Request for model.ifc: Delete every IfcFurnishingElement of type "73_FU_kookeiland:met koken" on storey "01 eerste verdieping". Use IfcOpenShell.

First a look at what the model holds.

```python
import ifcopenshell
import ifcopenshell.util.element

model = ifcopenshell.open("model.ifc")
print(model.schema)
storey = next(s for s in model.by_type("IfcBuildingStorey") if s.Name == "01 eerste verdieping")
furniture = [e for e in ifcopenshell.util.element.get_decomposition(storey) if e.is_a("IfcFurnishingElement")]
seen = {}
for e in furniture:
    element_type = ifcopenshell.util.element.get_type(e)
    name = element_type.Name if element_type not in (None, e) else None
    seen[name] = seen.get(name, 0) + 1
for name, count in sorted(seen.items(), key=str):
    print(count, "x", name)
```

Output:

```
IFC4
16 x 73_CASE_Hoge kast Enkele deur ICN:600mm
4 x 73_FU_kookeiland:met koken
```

```python
import ifcopenshell
import ifcopenshell.api.root
import ifcopenshell.util.element

model = ifcopenshell.open("model.ifc")

storey = next(s for s in model.by_type("IfcBuildingStorey") if s.Name == "01 eerste verdieping")
furniture = [e for e in ifcopenshell.util.element.get_decomposition(storey) if e.is_a("IfcFurnishingElement")]
targets = [e for e in furniture if (t := ifcopenshell.util.element.get_type(e)) not in (None, e) and t.Name == "73_FU_kookeiland:met koken"]

for e in targets:
    ifcopenshell.api.root.remove_product(model, product=e)
print(len(targets), "removed")

model.write("model_v2.ifc")
```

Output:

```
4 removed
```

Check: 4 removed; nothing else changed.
